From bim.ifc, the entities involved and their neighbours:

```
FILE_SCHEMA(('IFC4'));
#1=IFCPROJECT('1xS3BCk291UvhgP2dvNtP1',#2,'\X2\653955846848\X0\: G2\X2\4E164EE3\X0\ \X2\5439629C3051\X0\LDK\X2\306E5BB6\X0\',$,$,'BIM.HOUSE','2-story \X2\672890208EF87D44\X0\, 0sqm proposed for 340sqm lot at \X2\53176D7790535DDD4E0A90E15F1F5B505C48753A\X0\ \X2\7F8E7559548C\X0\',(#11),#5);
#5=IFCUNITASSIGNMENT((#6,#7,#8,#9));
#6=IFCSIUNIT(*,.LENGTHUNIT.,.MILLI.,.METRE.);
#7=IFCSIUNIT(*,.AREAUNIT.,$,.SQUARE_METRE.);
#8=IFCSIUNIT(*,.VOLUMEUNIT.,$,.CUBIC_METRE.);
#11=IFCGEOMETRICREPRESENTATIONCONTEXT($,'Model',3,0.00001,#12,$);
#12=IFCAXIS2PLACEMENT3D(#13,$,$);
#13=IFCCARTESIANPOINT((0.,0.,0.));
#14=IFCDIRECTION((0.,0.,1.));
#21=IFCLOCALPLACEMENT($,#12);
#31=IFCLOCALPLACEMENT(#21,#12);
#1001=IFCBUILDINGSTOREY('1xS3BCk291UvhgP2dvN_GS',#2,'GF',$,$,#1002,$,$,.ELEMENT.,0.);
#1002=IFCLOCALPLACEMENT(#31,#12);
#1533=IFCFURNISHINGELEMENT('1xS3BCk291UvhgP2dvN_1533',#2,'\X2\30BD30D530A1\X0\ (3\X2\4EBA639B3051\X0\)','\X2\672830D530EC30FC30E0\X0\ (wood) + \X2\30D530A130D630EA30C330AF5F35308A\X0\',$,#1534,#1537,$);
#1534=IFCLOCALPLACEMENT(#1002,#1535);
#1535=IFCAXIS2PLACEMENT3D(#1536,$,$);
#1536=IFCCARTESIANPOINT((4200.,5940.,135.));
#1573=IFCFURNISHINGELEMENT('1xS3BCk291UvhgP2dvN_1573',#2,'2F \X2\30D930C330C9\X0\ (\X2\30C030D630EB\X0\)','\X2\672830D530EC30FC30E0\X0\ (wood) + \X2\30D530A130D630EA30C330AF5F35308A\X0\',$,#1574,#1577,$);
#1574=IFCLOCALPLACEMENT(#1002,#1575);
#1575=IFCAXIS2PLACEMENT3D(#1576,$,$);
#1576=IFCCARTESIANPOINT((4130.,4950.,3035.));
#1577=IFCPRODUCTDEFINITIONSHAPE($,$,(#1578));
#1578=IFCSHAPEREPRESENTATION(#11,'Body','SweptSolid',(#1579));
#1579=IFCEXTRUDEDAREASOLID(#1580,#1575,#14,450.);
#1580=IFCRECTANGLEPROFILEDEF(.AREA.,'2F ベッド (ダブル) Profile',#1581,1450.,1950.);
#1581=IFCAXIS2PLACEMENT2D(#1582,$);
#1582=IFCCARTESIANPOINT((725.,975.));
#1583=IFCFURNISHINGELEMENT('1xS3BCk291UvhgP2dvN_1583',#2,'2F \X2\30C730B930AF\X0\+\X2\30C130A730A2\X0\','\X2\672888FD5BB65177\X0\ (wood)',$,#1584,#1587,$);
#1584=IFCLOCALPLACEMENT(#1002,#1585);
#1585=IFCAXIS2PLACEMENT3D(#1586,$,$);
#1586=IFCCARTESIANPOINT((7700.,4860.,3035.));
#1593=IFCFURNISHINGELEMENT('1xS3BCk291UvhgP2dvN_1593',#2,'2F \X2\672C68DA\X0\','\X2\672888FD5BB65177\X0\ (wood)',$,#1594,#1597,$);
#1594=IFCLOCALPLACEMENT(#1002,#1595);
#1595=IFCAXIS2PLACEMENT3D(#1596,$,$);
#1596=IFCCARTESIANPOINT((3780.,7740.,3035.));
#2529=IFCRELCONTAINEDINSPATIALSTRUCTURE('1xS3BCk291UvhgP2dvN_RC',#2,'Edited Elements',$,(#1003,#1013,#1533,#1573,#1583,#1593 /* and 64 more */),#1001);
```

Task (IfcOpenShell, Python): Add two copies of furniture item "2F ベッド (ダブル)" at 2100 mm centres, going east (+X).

```python
import numpy as np
import ifcopenshell
import ifcopenshell.api.geometry
import ifcopenshell.api.root
import ifcopenshell.util.element
import ifcopenshell.util.placement

model = ifcopenshell.open("bim.ifc")


def reuse_history(source, copy):
    """copy_class also copies each property set's owner history, people and application; keep the originals."""
    for rel in copy.IsDefinedBy:
        if rel.is_a("IfcRelDefinesByProperties") and (history := rel.RelatingPropertyDefinition.OwnerHistory):
            rel.RelatingPropertyDefinition.OwnerHistory = source.OwnerHistory
            ifcopenshell.util.element.remove_deep2(model, history)


source = model.by_id(1573)
base = ifcopenshell.util.placement.get_local_placement(source.ObjectPlacement)
step = np.array([1.0, 0.0, 0.0]) * 2100.0

for i in range(1, 3):
    copy = ifcopenshell.api.root.copy_class(model, product=source)
    copy.Representation = ifcopenshell.util.element.copy_deep(
        model, source.Representation, exclude=["IfcGeometricRepresentationContext", "IfcRepresentationMap"]
    )
    reuse_history(source, copy)
    matrix = base.copy()
    matrix[:3, 3] += i * step
    print("added at", matrix[:3, 3].round(3) + 0.0)
    ifcopenshell.api.geometry.edit_object_placement(model, product=copy, matrix=matrix, is_si=False)

model.write("bim_updated.ifc")
```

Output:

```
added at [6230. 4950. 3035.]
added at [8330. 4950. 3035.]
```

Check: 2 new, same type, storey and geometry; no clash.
